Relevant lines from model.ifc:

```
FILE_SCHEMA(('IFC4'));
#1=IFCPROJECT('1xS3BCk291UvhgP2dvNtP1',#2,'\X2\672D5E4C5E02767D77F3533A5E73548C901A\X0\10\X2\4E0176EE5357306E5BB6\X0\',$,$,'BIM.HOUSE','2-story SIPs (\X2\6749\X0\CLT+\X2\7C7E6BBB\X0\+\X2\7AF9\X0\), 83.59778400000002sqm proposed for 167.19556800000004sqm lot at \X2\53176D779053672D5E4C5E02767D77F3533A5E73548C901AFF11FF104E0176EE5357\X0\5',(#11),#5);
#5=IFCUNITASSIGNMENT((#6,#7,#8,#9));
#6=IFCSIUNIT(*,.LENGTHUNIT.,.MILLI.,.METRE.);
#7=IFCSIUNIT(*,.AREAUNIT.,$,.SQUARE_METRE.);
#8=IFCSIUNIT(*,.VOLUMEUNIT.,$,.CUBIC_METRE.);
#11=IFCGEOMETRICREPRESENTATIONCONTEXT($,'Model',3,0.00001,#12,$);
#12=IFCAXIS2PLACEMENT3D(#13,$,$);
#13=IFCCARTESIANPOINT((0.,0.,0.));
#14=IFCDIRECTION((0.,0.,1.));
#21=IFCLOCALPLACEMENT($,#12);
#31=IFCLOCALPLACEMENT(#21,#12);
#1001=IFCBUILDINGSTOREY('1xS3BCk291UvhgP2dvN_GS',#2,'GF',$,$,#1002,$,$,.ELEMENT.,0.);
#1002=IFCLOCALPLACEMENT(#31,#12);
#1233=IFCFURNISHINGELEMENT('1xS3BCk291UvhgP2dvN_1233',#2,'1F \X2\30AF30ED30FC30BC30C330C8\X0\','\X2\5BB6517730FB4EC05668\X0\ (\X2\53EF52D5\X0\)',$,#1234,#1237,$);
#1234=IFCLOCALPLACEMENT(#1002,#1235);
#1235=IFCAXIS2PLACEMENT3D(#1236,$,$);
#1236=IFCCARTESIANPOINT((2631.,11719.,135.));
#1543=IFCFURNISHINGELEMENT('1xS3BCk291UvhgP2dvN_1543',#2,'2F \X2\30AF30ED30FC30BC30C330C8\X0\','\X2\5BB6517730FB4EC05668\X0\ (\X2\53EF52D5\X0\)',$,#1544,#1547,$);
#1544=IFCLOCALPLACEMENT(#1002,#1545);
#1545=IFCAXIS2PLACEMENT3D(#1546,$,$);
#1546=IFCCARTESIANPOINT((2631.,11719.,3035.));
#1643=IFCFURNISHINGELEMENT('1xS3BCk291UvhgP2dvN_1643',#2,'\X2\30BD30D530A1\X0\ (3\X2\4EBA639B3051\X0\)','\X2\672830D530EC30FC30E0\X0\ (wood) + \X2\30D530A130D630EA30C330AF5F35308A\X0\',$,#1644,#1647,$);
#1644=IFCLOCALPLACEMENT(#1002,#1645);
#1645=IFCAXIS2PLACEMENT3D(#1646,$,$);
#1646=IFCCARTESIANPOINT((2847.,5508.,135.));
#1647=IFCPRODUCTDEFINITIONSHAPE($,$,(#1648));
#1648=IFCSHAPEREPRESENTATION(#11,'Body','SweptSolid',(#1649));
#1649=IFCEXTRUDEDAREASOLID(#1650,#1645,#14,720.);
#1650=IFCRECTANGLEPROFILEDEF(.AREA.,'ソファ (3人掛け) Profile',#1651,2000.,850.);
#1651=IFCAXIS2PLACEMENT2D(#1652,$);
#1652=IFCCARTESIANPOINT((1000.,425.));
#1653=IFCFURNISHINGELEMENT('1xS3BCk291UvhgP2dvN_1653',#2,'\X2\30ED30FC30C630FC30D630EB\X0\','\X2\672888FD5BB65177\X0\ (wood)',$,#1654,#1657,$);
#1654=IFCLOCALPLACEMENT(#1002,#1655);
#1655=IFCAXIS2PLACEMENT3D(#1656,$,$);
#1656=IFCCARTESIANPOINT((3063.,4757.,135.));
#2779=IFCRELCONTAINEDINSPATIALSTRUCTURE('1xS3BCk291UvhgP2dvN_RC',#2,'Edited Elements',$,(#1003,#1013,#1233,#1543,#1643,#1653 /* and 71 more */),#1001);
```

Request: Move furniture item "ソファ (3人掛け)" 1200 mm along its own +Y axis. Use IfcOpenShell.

```python
import ifcopenshell
import ifcopenshell.api.geometry
import ifcopenshell.util.placement
import ifcopenshell.util.unit

model = ifcopenshell.open("model.ifc")
unit_scale = ifcopenshell.util.unit.calculate_unit_scale(model)

item = model.by_id(1643)
matrix = ifcopenshell.util.placement.get_local_placement(item.ObjectPlacement)
matrix[:3, 3] += matrix[:3, 1] * 1.2 / unit_scale
ifcopenshell.api.geometry.edit_object_placement(model, product=item, matrix=matrix, is_si=False)

print(ifcopenshell.util.placement.get_local_placement(item.ObjectPlacement).round(3) + 0.0)

model.write("model-out.ifc")
```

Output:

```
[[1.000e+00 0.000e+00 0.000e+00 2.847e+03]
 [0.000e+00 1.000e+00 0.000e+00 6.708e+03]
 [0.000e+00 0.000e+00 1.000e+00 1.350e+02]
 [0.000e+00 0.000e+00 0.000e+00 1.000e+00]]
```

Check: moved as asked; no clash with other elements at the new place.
